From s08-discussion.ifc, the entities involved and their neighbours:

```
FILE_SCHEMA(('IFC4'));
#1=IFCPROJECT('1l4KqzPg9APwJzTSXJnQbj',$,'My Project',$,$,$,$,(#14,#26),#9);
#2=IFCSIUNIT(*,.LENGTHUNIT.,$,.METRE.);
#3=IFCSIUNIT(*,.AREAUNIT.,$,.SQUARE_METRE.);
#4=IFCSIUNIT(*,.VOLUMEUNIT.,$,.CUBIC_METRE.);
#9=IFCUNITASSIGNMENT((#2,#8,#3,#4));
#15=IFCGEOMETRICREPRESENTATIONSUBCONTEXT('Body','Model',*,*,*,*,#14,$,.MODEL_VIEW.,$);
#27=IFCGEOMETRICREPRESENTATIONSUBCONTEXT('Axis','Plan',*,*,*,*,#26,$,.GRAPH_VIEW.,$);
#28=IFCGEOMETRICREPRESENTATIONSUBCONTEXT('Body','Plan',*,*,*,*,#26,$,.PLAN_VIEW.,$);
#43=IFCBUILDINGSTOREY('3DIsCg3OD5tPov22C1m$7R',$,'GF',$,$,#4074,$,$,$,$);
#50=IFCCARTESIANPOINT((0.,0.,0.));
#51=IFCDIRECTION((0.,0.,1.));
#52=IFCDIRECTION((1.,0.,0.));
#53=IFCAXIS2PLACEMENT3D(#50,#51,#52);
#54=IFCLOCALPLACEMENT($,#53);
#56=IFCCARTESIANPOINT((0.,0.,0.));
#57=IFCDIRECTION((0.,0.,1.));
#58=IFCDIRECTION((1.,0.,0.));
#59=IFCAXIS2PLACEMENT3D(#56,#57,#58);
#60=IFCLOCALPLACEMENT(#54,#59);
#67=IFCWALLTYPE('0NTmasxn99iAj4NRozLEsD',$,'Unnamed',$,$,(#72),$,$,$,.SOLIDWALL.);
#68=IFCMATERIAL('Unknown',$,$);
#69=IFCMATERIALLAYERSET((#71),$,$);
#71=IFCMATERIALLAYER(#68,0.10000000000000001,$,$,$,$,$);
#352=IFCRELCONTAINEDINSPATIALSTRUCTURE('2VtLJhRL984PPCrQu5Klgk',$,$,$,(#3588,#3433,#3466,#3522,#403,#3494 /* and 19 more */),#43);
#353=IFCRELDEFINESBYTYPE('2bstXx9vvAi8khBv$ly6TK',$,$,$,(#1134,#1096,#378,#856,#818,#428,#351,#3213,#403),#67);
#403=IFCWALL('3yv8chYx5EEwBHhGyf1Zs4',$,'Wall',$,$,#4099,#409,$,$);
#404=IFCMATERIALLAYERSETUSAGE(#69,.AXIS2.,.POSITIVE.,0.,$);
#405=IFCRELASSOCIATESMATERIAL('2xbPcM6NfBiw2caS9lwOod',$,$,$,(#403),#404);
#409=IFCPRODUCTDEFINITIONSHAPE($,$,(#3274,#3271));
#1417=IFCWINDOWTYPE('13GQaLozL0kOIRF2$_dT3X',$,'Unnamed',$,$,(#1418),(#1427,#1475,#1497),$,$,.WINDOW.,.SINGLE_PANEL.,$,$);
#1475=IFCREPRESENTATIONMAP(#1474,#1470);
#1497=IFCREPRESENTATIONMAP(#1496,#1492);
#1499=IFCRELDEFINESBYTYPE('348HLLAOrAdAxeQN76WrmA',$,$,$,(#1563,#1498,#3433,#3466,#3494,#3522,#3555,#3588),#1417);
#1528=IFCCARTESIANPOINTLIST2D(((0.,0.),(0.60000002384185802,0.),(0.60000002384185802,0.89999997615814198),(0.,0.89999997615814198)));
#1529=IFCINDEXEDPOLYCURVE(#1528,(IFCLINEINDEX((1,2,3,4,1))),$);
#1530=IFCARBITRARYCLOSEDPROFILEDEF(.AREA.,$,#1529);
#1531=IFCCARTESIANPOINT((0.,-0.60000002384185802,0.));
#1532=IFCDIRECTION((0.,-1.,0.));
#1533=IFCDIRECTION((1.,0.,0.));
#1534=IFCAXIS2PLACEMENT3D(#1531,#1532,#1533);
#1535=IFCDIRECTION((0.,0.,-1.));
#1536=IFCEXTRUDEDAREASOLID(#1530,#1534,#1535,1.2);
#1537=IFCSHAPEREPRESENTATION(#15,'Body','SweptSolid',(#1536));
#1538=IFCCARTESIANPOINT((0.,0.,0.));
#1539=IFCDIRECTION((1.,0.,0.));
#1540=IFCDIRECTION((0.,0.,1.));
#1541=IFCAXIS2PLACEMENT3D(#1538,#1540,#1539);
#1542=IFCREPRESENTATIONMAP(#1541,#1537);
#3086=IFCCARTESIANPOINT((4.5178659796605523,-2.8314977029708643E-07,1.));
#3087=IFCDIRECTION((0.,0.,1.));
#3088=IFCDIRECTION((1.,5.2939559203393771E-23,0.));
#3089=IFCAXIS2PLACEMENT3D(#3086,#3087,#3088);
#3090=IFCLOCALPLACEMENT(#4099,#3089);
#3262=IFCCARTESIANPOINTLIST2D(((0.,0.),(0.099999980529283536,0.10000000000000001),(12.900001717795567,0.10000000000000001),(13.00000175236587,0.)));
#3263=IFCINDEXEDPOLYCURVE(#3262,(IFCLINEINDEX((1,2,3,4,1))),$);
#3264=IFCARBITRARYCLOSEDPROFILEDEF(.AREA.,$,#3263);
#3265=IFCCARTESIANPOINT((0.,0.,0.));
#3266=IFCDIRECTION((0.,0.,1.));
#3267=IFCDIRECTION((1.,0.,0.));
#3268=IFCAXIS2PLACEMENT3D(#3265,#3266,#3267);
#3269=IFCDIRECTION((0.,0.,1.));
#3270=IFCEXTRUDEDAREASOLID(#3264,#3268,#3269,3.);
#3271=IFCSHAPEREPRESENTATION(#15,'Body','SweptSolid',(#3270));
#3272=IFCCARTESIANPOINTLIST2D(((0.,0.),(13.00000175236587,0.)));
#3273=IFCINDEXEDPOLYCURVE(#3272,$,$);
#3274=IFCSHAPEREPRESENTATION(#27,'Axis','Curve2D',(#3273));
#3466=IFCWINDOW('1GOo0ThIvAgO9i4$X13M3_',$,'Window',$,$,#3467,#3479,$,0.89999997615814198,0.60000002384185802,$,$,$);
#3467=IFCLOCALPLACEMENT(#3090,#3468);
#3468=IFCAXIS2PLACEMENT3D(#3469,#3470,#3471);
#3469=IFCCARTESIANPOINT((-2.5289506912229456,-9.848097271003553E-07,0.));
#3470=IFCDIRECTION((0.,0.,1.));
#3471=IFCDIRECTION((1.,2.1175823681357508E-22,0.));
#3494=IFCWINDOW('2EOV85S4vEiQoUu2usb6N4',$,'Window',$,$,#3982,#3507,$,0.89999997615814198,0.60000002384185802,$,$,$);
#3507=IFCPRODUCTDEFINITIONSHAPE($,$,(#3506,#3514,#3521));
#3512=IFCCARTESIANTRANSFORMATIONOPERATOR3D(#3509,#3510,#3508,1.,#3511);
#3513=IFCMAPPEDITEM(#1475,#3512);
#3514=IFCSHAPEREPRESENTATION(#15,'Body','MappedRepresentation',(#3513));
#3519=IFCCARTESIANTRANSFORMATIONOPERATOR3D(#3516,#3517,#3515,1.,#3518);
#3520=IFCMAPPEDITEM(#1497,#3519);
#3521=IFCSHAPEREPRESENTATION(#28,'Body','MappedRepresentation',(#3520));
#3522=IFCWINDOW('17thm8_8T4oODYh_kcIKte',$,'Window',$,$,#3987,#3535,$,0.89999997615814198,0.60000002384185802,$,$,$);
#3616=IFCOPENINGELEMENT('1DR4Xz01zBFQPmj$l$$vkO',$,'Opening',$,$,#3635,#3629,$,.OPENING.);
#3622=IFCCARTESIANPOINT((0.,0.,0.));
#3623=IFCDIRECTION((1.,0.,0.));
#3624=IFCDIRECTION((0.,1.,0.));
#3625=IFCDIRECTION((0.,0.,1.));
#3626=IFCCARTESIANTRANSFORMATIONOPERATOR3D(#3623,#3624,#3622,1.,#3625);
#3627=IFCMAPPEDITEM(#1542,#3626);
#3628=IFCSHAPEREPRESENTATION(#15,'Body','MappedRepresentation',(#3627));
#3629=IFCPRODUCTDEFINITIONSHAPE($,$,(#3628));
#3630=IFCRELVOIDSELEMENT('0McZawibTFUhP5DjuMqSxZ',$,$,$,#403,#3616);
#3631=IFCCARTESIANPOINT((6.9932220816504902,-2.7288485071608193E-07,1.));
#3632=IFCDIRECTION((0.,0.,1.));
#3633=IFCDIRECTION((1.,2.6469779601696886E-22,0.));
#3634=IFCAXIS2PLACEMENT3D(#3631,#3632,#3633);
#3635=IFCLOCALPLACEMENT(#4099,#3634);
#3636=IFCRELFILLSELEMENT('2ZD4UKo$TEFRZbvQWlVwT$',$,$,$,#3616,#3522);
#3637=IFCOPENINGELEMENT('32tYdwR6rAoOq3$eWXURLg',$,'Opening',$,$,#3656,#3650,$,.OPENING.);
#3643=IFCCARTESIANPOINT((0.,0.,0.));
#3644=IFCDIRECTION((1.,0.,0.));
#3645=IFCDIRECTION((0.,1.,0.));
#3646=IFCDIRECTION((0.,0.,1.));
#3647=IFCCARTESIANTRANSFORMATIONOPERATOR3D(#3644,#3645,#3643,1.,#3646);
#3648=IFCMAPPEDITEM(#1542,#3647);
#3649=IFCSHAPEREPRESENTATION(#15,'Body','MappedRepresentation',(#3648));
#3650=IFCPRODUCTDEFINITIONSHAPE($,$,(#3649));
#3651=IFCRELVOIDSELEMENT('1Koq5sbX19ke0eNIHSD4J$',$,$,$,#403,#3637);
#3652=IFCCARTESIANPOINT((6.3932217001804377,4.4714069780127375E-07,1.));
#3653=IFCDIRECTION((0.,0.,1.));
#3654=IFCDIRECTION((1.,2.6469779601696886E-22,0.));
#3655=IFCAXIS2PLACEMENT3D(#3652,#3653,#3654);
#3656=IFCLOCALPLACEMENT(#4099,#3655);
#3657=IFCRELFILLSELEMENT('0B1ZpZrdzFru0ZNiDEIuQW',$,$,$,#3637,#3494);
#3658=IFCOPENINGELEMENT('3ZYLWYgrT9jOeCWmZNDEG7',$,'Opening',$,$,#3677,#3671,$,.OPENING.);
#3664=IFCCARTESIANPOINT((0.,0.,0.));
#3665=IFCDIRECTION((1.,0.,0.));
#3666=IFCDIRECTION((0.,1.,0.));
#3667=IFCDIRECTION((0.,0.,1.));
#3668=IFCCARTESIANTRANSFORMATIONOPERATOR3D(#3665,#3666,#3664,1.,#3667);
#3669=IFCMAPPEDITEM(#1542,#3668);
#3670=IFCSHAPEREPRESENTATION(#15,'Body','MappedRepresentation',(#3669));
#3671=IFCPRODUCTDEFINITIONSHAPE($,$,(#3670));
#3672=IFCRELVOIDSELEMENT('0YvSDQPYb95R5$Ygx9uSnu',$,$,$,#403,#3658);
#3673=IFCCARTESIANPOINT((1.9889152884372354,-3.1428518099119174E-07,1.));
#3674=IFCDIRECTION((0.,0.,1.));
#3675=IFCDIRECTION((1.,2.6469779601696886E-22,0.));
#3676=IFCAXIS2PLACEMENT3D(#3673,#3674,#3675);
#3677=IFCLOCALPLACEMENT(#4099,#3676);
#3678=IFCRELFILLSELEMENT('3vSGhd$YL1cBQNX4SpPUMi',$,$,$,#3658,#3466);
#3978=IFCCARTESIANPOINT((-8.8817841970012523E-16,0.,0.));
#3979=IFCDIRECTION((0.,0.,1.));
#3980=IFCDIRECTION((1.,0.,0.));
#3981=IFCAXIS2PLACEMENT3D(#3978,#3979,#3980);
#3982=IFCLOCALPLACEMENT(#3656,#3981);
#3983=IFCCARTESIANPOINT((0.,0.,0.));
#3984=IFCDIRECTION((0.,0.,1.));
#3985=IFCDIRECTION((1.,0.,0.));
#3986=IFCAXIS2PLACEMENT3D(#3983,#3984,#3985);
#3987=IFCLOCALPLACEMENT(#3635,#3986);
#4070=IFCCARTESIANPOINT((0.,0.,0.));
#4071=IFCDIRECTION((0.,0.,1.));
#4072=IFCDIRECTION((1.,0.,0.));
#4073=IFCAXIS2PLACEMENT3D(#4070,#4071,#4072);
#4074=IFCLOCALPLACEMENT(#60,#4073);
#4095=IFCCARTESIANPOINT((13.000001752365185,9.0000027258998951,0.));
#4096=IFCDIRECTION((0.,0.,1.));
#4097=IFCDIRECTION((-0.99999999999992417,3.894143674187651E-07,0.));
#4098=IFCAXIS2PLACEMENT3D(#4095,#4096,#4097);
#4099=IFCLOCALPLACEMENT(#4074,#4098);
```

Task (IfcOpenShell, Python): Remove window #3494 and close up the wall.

```python
import ifcopenshell
import ifcopenshell.api.feature
import ifcopenshell.api.root
import ifcopenshell.geom
import ifcopenshell.util.shape

model = ifcopenshell.open("s08-discussion.ifc")
settings = ifcopenshell.geom.settings()


def volume(element):
    """Net volume in cubic metres, openings subtracted."""
    shape = ifcopenshell.geom.create_shape(settings, element)
    return ifcopenshell.util.shape.get_volume(shape.geometry)


window = model.by_id(3494)
opening = window.FillsVoids[0].RelatingOpeningElement
wall = opening.VoidsElements[0].RelatingBuildingElement
before = volume(wall)

ifcopenshell.api.root.remove_product(model, product=window)
ifcopenshell.api.feature.remove_feature(model, feature=opening)

after = volume(wall)

print(f"wall volume {before:.3f} -> {after:.3f} m3")

model.write("s08-discussion_v2.ifc")
```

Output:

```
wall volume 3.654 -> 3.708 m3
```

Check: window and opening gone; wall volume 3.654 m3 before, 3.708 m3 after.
